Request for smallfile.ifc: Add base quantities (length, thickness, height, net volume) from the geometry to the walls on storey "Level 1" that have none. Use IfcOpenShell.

First a look at what the model holds.

```python
import ifcopenshell
import ifcopenshell.util.element
import ifcopenshell.util.unit

model = ifcopenshell.open("smallfile.ifc")
print(model.schema)
for unit_type in ("LENGTHUNIT", "AREAUNIT", "VOLUMEUNIT"):
    print(unit_type, ifcopenshell.util.unit.calculate_unit_scale(model, unit_type))
storey = next(s for s in model.by_type("IfcBuildingStorey") if s.Name == "Level 1")
walls = [e for e in ifcopenshell.util.element.get_decomposition(storey) if e.is_a("IfcWall")]
for e in sorted(walls, key=lambda e: e.id()):
    print(e.id(), e.is_a(), e.Name, list(ifcopenshell.util.element.get_psets(e, qtos_only=True)), sep=" | ")
```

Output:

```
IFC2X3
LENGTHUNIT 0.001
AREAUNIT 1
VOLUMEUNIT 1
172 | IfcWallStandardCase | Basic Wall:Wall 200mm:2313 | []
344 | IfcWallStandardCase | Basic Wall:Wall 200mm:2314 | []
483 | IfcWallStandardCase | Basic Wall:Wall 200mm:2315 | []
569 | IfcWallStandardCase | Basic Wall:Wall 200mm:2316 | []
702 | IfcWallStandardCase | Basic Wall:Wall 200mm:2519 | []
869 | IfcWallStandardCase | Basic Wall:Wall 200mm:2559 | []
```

```python
import ifcopenshell
import ifcopenshell.api.pset
import ifcopenshell.geom
import ifcopenshell.util.element
import ifcopenshell.util.shape
import ifcopenshell.util.unit

model = ifcopenshell.open("smallfile.ifc")
unit_scale = ifcopenshell.util.unit.calculate_unit_scale(model)
volume_scale = ifcopenshell.util.unit.calculate_unit_scale(model, "VOLUMEUNIT")
settings = ifcopenshell.geom.settings()

storey = next(s for s in model.by_type("IfcBuildingStorey") if s.Name == "Level 1")
walls = [e for e in ifcopenshell.util.element.get_decomposition(storey) if e.is_a("IfcWall")]

for e in sorted(walls, key=lambda e: e.id()):
    if ifcopenshell.util.element.get_psets(e, qtos_only=True, should_inherit=False):
        continue
    # Geometry comes back in metres, in the element's own axes.
    shape = ifcopenshell.geom.create_shape(settings, e)
    values = {
        "Length": ifcopenshell.util.shape.get_x(shape.geometry) / unit_scale,
        "Width": ifcopenshell.util.shape.get_y(shape.geometry) / unit_scale,
        "Height": ifcopenshell.util.shape.get_z(shape.geometry) / unit_scale,
        "NetVolume": ifcopenshell.util.shape.get_volume(shape.geometry) / volume_scale,
    }
    qto = ifcopenshell.api.pset.add_qto(model, product=e, name="BaseQuantities")
    ifcopenshell.api.pset.edit_qto(model, qto=qto, properties=values)
    print(e.id(), {k: round(v, 3) for k, v in values.items()})

model.write("smallfile_rev.ifc")
```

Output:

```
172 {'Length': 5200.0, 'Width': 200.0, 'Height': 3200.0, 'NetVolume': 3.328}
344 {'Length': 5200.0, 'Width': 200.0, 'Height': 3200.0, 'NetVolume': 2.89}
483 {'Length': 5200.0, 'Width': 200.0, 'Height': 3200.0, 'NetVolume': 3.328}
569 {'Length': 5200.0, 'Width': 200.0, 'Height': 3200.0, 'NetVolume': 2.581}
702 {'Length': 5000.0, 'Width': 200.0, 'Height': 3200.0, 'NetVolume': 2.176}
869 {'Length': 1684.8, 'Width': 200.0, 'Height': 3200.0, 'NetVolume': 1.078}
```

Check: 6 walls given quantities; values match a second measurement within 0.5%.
